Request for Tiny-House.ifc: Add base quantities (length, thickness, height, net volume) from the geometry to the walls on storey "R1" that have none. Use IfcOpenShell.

First a look at what the model holds.

```python
import ifcopenshell
import ifcopenshell.util.element
import ifcopenshell.util.unit

model = ifcopenshell.open("Tiny-House.ifc")
print(model.schema)
for unit_type in ("LENGTHUNIT", "AREAUNIT", "VOLUMEUNIT"):
    print(unit_type, ifcopenshell.util.unit.calculate_unit_scale(model, unit_type))
storey = next(s for s in model.by_type("IfcBuildingStorey") if s.Name == "R1")
walls = [e for e in ifcopenshell.util.element.get_decomposition(storey) if e.is_a("IfcWall")]
for e in sorted(walls, key=lambda e: e.id()):
    print(e.id(), e.is_a(), e.Name, list(ifcopenshell.util.element.get_psets(e, qtos_only=True)), sep=" | ")
```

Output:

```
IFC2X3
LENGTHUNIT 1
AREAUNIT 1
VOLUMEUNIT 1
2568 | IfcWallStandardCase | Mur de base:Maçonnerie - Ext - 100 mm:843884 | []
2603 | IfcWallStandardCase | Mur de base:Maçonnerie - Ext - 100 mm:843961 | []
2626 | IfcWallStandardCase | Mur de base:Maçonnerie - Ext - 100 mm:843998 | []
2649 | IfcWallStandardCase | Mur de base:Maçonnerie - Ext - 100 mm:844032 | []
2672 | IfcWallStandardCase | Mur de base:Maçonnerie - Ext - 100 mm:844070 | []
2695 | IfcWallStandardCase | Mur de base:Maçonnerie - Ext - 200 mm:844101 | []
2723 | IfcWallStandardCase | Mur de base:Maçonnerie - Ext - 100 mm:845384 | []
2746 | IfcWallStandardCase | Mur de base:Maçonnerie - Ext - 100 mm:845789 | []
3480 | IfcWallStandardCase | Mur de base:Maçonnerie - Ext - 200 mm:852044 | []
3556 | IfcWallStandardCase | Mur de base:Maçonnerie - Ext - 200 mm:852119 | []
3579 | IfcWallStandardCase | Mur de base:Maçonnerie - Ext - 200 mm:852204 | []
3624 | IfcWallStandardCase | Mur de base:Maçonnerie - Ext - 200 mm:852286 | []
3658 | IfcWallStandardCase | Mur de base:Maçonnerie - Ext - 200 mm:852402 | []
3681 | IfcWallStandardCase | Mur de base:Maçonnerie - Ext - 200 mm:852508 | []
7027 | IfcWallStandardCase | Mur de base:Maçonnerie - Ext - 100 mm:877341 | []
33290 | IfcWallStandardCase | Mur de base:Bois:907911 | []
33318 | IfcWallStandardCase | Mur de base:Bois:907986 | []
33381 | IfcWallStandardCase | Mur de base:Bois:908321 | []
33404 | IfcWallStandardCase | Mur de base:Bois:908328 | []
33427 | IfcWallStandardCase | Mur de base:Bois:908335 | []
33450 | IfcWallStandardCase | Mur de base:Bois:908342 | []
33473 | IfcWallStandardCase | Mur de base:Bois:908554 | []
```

```python
import ifcopenshell
import ifcopenshell.api.pset
import ifcopenshell.geom
import ifcopenshell.util.element
import ifcopenshell.util.shape
import ifcopenshell.util.unit

model = ifcopenshell.open("Tiny-House.ifc")
unit_scale = ifcopenshell.util.unit.calculate_unit_scale(model)
volume_scale = ifcopenshell.util.unit.calculate_unit_scale(model, "VOLUMEUNIT")
settings = ifcopenshell.geom.settings()

storey = next(s for s in model.by_type("IfcBuildingStorey") if s.Name == "R1")
walls = [e for e in ifcopenshell.util.element.get_decomposition(storey) if e.is_a("IfcWall")]

for e in sorted(walls, key=lambda e: e.id()):
    if ifcopenshell.util.element.get_psets(e, qtos_only=True, should_inherit=False):
        continue
    # Geometry comes back in metres, in the element's own axes.
    shape = ifcopenshell.geom.create_shape(settings, e)
    values = {
        "Length": ifcopenshell.util.shape.get_x(shape.geometry) / unit_scale,
        "Width": ifcopenshell.util.shape.get_y(shape.geometry) / unit_scale,
        "Height": ifcopenshell.util.shape.get_z(shape.geometry) / unit_scale,
        "NetVolume": ifcopenshell.util.shape.get_volume(shape.geometry) / volume_scale,
    }
    qto = ifcopenshell.api.pset.add_qto(model, product=e, name="BaseQuantities")
    ifcopenshell.api.pset.edit_qto(model, qto=qto, properties=values)
    print(e.id(), {k: round(v, 3) for k, v in values.items()})

model.write("Tiny-House_edited.ifc")
```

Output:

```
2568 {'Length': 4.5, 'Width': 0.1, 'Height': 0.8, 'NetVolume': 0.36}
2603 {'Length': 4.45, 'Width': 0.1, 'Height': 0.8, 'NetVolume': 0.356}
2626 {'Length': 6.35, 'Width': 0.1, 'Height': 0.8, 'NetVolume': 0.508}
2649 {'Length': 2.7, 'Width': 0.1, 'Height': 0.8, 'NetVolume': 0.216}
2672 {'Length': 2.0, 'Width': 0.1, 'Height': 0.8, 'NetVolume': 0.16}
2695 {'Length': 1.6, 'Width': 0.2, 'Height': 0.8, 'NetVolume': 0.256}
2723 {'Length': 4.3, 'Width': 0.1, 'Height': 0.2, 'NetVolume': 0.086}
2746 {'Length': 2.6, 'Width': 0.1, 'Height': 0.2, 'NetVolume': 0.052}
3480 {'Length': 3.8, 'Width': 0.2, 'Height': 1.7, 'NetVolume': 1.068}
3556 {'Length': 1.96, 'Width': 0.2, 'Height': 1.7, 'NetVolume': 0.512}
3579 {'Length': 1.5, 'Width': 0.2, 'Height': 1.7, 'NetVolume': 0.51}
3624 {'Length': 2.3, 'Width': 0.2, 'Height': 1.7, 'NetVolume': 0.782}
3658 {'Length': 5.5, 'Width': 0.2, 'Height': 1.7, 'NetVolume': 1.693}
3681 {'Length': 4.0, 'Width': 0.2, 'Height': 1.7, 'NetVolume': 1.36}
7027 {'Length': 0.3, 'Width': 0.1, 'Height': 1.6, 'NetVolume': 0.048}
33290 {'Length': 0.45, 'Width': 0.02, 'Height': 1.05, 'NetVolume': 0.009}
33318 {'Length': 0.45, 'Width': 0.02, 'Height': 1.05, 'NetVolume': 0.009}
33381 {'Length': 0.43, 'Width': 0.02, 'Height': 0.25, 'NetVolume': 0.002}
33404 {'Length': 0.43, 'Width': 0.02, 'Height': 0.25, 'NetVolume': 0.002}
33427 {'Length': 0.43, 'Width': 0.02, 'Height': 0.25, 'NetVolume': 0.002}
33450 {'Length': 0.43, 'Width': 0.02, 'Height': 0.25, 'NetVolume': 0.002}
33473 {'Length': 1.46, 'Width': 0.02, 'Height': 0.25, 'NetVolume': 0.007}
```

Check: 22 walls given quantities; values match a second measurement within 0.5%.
